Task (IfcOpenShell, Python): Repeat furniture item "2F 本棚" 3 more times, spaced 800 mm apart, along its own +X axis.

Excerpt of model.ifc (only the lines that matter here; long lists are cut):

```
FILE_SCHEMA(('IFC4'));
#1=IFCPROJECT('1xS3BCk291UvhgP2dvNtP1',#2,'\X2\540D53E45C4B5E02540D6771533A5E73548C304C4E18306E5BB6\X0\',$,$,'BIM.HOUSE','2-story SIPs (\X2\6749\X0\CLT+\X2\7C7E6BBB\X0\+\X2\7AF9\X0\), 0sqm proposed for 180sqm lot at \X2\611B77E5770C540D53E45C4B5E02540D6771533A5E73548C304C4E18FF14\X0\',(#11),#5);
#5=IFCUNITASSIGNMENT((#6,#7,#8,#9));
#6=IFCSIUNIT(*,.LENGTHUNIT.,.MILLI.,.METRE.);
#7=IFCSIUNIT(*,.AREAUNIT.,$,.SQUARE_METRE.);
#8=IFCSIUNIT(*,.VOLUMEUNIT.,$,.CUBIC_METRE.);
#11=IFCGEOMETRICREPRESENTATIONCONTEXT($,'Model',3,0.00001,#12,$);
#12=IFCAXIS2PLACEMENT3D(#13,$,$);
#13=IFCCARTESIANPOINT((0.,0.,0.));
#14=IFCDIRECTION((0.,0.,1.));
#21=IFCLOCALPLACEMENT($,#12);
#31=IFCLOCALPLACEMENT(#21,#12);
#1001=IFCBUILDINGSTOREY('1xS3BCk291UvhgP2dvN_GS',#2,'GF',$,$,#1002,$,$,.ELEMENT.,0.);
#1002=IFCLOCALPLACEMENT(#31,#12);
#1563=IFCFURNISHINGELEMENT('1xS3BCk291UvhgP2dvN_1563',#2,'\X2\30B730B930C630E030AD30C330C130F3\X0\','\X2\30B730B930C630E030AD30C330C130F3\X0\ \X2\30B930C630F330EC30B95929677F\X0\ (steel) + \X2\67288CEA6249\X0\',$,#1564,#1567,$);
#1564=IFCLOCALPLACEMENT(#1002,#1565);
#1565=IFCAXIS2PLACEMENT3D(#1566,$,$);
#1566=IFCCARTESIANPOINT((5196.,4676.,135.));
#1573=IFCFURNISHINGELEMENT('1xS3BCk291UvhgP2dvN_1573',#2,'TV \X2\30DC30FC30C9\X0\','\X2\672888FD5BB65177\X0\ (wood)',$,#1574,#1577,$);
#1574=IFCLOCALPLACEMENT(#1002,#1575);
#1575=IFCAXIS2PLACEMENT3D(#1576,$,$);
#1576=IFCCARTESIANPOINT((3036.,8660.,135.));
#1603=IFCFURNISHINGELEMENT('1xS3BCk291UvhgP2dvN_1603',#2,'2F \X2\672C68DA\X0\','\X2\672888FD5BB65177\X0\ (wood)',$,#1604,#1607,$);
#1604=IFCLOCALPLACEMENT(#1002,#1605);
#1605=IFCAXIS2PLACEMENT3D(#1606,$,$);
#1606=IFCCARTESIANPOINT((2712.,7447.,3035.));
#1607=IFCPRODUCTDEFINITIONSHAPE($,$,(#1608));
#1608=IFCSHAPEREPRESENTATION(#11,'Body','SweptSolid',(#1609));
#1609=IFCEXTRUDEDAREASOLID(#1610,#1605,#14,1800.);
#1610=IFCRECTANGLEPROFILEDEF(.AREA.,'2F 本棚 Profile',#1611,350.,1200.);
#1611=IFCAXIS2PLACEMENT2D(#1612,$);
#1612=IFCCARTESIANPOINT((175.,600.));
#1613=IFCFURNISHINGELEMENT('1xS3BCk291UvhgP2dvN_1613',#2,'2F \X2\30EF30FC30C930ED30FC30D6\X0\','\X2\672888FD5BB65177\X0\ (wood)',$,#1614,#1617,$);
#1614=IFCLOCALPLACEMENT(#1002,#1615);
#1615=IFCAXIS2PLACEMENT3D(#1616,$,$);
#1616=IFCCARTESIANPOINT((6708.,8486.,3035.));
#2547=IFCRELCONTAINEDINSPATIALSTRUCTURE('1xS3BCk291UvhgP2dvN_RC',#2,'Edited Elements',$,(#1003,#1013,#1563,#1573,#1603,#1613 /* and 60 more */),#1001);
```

```python
import ifcopenshell
import ifcopenshell.api.geometry
import ifcopenshell.api.root
import ifcopenshell.util.element
import ifcopenshell.util.placement
import ifcopenshell.util.unit

model = ifcopenshell.open("model.ifc")
unit_scale = ifcopenshell.util.unit.calculate_unit_scale(model)


def reuse_history(source, copy):
    """copy_class also copies each property set's owner history, people and application; keep the originals."""
    for rel in copy.IsDefinedBy:
        if rel.is_a("IfcRelDefinesByProperties") and (history := rel.RelatingPropertyDefinition.OwnerHistory):
            rel.RelatingPropertyDefinition.OwnerHistory = source.OwnerHistory
            ifcopenshell.util.element.remove_deep2(model, history)


source = model.by_guid("1xS3BCk291UvhgP2dvN_1603")
base = ifcopenshell.util.placement.get_local_placement(source.ObjectPlacement)
step = base[:3, 0] * 0.8 / unit_scale

for i in range(1, 4):
    copy = ifcopenshell.api.root.copy_class(model, product=source)
    copy.Representation = ifcopenshell.util.element.copy_deep(
        model, source.Representation, exclude=["IfcGeometricRepresentationContext", "IfcRepresentationMap"]
    )
    reuse_history(source, copy)
    matrix = base.copy()
    matrix[:3, 3] += i * step
    print("added at", matrix[:3, 3].round(3) + 0.0)
    ifcopenshell.api.geometry.edit_object_placement(model, product=copy, matrix=matrix, is_si=False)

model.write("model_v2.ifc")
```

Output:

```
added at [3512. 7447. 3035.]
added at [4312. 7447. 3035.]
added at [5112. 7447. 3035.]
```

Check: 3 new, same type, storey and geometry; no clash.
